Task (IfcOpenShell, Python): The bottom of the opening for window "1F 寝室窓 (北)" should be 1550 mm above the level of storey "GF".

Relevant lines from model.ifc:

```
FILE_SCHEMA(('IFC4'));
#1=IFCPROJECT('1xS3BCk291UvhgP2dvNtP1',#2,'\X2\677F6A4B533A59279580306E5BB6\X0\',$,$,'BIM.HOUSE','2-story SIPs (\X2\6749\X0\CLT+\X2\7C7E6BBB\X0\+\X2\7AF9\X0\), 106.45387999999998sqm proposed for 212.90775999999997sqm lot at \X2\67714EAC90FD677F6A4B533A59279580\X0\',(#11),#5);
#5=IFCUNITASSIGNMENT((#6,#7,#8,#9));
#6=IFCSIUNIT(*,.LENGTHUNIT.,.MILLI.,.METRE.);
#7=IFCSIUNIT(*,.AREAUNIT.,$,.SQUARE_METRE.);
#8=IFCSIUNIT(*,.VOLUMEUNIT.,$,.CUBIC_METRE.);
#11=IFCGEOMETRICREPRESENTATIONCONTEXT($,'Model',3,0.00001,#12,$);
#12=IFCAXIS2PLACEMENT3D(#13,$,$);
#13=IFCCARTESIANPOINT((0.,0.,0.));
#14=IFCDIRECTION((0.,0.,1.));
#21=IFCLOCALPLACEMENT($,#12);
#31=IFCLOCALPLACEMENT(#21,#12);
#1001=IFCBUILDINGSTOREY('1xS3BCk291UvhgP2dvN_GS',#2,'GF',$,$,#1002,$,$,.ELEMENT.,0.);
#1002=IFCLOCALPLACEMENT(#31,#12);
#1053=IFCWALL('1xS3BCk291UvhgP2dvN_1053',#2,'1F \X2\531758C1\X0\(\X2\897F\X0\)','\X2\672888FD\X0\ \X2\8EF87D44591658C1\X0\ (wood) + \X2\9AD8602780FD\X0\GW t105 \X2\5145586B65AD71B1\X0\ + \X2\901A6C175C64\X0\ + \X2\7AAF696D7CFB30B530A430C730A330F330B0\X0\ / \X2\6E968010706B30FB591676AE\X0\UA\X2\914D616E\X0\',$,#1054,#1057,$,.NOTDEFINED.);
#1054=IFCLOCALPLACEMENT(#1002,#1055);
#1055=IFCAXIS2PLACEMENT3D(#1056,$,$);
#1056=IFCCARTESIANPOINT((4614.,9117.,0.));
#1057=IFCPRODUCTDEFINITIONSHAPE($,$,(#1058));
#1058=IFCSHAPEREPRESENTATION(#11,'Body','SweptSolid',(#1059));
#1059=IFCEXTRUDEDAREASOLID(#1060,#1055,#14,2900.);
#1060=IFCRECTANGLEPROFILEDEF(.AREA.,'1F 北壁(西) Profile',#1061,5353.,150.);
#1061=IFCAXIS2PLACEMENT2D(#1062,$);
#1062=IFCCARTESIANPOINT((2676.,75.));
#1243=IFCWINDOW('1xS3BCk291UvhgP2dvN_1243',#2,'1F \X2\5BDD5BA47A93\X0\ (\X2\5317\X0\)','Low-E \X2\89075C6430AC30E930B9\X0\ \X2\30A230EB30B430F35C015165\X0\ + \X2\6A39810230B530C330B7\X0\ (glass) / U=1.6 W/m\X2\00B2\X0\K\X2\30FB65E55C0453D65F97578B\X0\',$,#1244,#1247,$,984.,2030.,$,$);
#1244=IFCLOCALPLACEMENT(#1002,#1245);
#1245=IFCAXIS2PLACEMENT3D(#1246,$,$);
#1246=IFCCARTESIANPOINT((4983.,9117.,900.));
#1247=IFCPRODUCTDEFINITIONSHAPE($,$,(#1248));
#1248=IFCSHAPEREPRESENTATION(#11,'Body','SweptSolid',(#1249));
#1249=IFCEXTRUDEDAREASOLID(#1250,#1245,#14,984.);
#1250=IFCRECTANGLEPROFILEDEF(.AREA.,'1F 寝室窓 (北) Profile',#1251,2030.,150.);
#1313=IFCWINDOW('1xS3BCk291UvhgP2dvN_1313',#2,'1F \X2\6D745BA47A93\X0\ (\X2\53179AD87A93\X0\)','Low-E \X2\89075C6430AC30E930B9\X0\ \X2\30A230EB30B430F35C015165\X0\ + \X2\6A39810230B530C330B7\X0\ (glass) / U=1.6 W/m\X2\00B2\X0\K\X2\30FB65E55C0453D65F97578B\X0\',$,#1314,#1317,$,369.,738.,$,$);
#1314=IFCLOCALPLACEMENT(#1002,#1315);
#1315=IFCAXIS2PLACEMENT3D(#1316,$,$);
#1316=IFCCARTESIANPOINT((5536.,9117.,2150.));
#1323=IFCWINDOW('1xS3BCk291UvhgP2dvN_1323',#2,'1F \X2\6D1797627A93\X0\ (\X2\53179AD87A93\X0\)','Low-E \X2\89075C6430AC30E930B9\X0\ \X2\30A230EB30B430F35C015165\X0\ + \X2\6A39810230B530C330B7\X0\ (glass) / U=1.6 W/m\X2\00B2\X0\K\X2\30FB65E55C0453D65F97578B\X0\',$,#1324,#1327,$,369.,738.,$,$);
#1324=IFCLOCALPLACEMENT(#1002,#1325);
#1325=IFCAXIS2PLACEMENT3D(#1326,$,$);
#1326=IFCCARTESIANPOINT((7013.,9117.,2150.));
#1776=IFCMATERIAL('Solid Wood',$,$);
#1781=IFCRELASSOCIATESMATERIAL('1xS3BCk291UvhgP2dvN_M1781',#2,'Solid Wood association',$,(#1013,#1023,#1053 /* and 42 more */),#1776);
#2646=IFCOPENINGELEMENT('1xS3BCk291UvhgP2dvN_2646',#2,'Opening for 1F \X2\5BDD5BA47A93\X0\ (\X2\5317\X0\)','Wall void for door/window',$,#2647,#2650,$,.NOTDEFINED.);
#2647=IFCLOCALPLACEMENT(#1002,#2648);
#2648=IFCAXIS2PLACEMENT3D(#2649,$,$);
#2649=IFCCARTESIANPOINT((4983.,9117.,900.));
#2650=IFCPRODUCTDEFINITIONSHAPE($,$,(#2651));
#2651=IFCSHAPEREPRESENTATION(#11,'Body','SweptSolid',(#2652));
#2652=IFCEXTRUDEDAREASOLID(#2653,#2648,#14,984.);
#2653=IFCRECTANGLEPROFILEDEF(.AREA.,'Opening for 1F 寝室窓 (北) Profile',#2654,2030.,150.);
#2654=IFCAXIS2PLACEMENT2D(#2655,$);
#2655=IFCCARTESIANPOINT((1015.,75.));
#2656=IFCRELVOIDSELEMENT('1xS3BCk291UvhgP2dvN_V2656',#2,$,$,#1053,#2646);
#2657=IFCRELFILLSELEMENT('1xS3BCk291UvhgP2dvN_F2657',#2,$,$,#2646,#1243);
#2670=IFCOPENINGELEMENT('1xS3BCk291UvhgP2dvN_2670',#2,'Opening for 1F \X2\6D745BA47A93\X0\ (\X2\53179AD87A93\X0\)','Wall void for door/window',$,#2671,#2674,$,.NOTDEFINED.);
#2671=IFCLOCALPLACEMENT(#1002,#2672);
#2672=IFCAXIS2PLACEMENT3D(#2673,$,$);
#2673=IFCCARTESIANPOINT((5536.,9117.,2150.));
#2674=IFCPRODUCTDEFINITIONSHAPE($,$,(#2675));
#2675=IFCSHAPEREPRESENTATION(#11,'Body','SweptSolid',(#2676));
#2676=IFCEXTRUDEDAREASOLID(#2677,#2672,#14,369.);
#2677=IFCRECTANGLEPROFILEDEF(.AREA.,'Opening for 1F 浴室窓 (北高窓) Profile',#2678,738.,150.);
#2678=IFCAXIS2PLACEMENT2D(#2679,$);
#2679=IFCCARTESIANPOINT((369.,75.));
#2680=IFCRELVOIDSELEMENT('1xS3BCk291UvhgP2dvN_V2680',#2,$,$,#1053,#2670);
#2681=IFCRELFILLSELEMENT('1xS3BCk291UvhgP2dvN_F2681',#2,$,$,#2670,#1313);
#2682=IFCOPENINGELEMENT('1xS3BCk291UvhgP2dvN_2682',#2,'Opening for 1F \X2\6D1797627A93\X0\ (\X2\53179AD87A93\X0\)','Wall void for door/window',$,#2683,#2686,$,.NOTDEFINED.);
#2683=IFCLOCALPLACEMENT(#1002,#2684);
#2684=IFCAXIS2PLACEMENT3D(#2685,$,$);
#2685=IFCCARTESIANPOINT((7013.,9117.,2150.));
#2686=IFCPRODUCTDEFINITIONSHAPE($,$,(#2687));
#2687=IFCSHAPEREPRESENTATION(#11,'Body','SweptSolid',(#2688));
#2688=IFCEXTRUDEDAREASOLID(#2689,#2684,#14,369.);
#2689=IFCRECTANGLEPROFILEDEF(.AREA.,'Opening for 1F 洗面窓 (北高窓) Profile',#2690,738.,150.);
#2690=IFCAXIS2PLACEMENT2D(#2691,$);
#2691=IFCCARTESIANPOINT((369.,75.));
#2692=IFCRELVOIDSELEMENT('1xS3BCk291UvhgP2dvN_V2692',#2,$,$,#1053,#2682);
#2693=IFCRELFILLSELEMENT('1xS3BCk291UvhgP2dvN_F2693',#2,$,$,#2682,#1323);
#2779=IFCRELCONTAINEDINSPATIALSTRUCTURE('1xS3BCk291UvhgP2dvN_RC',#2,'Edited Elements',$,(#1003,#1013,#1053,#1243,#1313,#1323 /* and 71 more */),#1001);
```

```python
import numpy as np
import ifcopenshell
import ifcopenshell.api.geometry
import ifcopenshell.geom
import ifcopenshell.util.element
import ifcopenshell.util.placement
import ifcopenshell.util.shape
import ifcopenshell.util.unit

model = ifcopenshell.open("model.ifc")
unit_scale = ifcopenshell.util.unit.calculate_unit_scale(model)

window = model.by_guid("1xS3BCk291UvhgP2dvN_1243")
opening = window.FillsVoids[0].RelatingOpeningElement
storey = ifcopenshell.util.element.get_container(window, ifc_class="IfcBuildingStorey")
level = ifcopenshell.util.placement.get_local_placement(storey.ObjectPlacement)[2, 3]

# The opening's origin need not be at the sill, so measure its lowest point.
shape = ifcopenshell.geom.create_shape(ifcopenshell.geom.settings(), opening)
bottom = ifcopenshell.util.shape.get_shape_bottom_elevation(shape, shape.geometry) / unit_scale
dz = level + 1.55 / unit_scale - bottom

shift = np.array([0.0, 0.0, dz])
# The window is not placed relative to its opening, so move both.
for product in (opening, window):
    matrix = ifcopenshell.util.placement.get_local_placement(product.ObjectPlacement)
    matrix[:3, 3] += shift
    ifcopenshell.api.geometry.edit_object_placement(model, product=product, matrix=matrix, is_si=False)

print(f"moved by {dz * unit_scale:+.3f} m")

model.write("model_rev.ifc")
```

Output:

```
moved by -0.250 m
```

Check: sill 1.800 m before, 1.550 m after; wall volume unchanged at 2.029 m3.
